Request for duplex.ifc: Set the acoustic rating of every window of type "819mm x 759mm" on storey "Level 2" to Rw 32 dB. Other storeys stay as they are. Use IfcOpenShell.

First a look at what the model holds.

```python
import ifcopenshell
import ifcopenshell.util.element

model = ifcopenshell.open("duplex.ifc")
print(model.schema)
storey = next(s for s in model.by_type("IfcBuildingStorey") if s.Name == "Level 2")
windows = [e for e in ifcopenshell.util.element.get_decomposition(storey) if e.is_a("IfcWindow")]
seen = {}
for e in windows:
    element_type = ifcopenshell.util.element.get_type(e)
    key = (element_type.Name if element_type != e and element_type else None, ifcopenshell.util.element.get_pset(e, "Pset_WindowCommon", "AcousticRating"))
    seen[key] = seen.get(key, 0) + 1
for (name, value), count in sorted(seen.items(), key=str):
    print(count, "x", name, "|", value)
```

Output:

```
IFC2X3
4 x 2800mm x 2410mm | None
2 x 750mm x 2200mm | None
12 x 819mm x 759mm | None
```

```python
import ifcopenshell
import ifcopenshell.api.pset
import ifcopenshell.util.element

model = ifcopenshell.open("duplex.ifc")

storey = next(s for s in model.by_type("IfcBuildingStorey") if s.Name == "Level 2")
windows = [e for e in ifcopenshell.util.element.get_decomposition(storey) if e.is_a("IfcWindow")]

count = 0
for e in windows:
    element_type = ifcopenshell.util.element.get_type(e)
    if element_type in (None, e) or element_type.Name != "819mm x 759mm":
        continue
    # add_pset returns the element's existing set when there is one.
    pset = ifcopenshell.api.pset.add_pset(model, product=e, name="Pset_WindowCommon")
    ifcopenshell.api.pset.edit_pset(model, pset=pset, properties={"AcousticRating": "Rw 32 dB"})
    count += 1

print(count, "windows updated")

model.write("duplex_v2.ifc")
```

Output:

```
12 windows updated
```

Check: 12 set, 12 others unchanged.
